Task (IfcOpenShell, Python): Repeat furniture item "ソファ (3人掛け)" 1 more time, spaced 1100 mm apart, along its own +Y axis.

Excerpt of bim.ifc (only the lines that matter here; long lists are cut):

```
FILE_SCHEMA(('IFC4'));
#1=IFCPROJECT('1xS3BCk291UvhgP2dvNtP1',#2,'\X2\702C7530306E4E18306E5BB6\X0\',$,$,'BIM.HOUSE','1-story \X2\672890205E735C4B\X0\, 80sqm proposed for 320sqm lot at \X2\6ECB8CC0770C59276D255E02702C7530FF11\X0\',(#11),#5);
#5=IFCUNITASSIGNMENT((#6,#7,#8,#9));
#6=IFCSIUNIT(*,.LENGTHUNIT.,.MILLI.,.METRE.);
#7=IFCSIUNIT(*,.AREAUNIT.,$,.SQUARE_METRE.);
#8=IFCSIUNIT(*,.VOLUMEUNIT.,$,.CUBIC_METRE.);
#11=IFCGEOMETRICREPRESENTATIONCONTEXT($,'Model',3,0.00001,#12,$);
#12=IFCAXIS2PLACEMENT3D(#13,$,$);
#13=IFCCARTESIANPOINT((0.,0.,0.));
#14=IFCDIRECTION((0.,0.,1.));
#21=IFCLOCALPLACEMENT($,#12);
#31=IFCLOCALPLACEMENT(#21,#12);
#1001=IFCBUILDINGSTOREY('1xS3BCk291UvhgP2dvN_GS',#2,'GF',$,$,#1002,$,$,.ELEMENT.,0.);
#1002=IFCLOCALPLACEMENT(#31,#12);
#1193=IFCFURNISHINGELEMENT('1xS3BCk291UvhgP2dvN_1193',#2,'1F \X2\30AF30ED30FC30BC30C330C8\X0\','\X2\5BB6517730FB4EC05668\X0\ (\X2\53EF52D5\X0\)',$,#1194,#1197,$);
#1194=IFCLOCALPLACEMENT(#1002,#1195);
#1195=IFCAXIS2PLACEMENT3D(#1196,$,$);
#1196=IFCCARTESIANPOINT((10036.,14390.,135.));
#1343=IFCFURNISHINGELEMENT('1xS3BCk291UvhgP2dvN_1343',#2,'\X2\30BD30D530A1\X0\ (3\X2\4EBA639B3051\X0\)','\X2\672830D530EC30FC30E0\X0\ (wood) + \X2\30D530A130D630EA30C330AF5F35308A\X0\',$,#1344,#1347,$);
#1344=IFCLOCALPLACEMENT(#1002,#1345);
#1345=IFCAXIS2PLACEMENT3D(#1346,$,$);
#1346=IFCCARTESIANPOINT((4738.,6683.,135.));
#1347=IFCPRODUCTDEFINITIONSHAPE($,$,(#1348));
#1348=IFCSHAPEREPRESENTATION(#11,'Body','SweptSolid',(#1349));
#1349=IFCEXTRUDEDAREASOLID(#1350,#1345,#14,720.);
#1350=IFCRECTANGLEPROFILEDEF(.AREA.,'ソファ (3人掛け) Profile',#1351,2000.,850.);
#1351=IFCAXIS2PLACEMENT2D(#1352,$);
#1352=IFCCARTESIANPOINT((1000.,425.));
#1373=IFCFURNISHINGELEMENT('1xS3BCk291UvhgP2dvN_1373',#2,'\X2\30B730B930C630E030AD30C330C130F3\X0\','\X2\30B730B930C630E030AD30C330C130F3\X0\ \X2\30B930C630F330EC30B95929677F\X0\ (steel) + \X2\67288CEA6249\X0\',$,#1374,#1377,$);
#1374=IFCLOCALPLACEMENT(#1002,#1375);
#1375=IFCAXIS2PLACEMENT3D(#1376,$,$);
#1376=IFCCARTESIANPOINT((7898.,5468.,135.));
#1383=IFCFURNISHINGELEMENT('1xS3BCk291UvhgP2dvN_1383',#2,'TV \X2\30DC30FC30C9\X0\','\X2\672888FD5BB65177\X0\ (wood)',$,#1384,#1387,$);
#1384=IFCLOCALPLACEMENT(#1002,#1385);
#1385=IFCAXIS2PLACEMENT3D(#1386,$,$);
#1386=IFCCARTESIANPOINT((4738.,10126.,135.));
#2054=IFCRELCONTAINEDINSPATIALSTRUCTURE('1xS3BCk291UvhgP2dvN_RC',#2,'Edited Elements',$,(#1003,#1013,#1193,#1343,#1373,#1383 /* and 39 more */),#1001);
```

```python
import ifcopenshell
import ifcopenshell.api.geometry
import ifcopenshell.api.root
import ifcopenshell.util.element
import ifcopenshell.util.placement
import ifcopenshell.util.unit

model = ifcopenshell.open("bim.ifc")
unit_scale = ifcopenshell.util.unit.calculate_unit_scale(model)


def reuse_history(source, copy):
    """copy_class also copies each property set's owner history, people and application; keep the originals."""
    for rel in copy.IsDefinedBy:
        if rel.is_a("IfcRelDefinesByProperties") and (history := rel.RelatingPropertyDefinition.OwnerHistory):
            rel.RelatingPropertyDefinition.OwnerHistory = source.OwnerHistory
            ifcopenshell.util.element.remove_deep2(model, history)


source = model.by_guid("1xS3BCk291UvhgP2dvN_1343")
base = ifcopenshell.util.placement.get_local_placement(source.ObjectPlacement)
step = base[:3, 1] * 1.1 / unit_scale

for i in range(1, 2):
    copy = ifcopenshell.api.root.copy_class(model, product=source)
    copy.Representation = ifcopenshell.util.element.copy_deep(
        model, source.Representation, exclude=["IfcGeometricRepresentationContext", "IfcRepresentationMap"]
    )
    reuse_history(source, copy)
    matrix = base.copy()
    matrix[:3, 3] += i * step
    print("added at", matrix[:3, 3].round(3) + 0.0)
    ifcopenshell.api.geometry.edit_object_placement(model, product=copy, matrix=matrix, is_si=False)

model.write("bim_v2.ifc")
```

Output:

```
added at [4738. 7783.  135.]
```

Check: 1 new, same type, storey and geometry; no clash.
